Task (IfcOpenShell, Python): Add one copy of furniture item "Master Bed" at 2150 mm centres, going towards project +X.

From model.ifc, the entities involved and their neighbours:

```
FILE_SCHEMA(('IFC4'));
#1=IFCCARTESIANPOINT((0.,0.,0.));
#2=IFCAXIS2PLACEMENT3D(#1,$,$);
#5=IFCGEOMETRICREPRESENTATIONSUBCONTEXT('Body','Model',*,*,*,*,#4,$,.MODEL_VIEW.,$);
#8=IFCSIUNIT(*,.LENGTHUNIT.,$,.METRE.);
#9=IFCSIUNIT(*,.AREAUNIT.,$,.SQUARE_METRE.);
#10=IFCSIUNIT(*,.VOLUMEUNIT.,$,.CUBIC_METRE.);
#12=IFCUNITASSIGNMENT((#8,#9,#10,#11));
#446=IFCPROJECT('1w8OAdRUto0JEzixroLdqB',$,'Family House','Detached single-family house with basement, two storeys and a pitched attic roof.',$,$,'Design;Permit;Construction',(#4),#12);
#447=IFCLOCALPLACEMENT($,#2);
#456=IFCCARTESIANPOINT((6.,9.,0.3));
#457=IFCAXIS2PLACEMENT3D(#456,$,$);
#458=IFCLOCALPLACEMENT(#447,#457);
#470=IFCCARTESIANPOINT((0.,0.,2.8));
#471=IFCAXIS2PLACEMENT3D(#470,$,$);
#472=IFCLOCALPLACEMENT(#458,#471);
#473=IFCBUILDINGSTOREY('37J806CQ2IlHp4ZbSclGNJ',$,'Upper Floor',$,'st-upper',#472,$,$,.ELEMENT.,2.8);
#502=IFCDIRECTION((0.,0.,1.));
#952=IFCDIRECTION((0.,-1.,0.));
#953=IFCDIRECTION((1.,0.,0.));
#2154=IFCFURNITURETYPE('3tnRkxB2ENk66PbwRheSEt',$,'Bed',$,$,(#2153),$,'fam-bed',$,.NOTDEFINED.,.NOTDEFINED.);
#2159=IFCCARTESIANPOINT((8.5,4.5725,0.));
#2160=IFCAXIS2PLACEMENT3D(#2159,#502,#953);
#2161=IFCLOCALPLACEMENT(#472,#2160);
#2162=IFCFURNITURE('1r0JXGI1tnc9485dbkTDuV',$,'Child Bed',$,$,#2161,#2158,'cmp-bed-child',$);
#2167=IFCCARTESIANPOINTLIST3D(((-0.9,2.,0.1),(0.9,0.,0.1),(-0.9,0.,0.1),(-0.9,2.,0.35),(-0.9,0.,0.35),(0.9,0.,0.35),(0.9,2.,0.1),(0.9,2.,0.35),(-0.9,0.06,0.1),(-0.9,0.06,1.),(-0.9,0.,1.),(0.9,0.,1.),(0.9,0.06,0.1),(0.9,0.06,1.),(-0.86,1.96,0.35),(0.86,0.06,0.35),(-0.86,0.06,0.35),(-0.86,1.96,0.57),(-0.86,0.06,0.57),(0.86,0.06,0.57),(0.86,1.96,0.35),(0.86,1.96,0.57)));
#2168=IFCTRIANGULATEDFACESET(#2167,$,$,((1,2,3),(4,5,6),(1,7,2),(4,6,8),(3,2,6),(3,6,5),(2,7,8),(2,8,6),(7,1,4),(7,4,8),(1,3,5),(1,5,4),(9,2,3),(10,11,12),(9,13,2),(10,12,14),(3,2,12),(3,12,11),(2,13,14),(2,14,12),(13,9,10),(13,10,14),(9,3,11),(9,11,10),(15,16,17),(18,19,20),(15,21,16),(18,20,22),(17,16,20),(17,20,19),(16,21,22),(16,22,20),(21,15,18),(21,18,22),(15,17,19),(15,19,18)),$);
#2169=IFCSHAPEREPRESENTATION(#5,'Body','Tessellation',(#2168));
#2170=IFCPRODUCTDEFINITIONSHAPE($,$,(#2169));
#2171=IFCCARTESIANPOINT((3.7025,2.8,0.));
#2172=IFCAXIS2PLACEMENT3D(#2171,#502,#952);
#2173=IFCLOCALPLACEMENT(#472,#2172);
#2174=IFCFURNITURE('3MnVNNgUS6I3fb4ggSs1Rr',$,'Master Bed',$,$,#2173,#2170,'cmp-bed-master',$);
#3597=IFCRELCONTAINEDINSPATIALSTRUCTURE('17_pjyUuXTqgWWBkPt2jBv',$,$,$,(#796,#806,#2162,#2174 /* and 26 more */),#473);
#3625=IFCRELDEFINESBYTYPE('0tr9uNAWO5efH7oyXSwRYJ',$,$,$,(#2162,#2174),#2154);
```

```python
import numpy as np
import ifcopenshell
import ifcopenshell.api.geometry
import ifcopenshell.api.root
import ifcopenshell.util.element
import ifcopenshell.util.placement
import ifcopenshell.util.unit

model = ifcopenshell.open("model.ifc")
unit_scale = ifcopenshell.util.unit.calculate_unit_scale(model)

source = model.by_guid("3MnVNNgUS6I3fb4ggSs1Rr")
base = ifcopenshell.util.placement.get_local_placement(source.ObjectPlacement)
step = np.array([1.0, 0.0, 0.0]) * 2.15 / unit_scale

for i in range(1, 2):
    copy = ifcopenshell.api.root.copy_class(model, product=source)
    copy.Representation = ifcopenshell.util.element.copy_deep(
        model, source.Representation, exclude=["IfcGeometricRepresentationContext", "IfcRepresentationMap"]
    )
    copy.Tag = None
    matrix = base.copy()
    matrix[:3, 3] += i * step
    print("added at", matrix[:3, 3].round(3) + 0.0)
    ifcopenshell.api.geometry.edit_object_placement(model, product=copy, matrix=matrix, is_si=False)

model.write("model_rev.ifc")
```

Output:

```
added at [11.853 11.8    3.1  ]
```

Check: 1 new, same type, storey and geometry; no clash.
